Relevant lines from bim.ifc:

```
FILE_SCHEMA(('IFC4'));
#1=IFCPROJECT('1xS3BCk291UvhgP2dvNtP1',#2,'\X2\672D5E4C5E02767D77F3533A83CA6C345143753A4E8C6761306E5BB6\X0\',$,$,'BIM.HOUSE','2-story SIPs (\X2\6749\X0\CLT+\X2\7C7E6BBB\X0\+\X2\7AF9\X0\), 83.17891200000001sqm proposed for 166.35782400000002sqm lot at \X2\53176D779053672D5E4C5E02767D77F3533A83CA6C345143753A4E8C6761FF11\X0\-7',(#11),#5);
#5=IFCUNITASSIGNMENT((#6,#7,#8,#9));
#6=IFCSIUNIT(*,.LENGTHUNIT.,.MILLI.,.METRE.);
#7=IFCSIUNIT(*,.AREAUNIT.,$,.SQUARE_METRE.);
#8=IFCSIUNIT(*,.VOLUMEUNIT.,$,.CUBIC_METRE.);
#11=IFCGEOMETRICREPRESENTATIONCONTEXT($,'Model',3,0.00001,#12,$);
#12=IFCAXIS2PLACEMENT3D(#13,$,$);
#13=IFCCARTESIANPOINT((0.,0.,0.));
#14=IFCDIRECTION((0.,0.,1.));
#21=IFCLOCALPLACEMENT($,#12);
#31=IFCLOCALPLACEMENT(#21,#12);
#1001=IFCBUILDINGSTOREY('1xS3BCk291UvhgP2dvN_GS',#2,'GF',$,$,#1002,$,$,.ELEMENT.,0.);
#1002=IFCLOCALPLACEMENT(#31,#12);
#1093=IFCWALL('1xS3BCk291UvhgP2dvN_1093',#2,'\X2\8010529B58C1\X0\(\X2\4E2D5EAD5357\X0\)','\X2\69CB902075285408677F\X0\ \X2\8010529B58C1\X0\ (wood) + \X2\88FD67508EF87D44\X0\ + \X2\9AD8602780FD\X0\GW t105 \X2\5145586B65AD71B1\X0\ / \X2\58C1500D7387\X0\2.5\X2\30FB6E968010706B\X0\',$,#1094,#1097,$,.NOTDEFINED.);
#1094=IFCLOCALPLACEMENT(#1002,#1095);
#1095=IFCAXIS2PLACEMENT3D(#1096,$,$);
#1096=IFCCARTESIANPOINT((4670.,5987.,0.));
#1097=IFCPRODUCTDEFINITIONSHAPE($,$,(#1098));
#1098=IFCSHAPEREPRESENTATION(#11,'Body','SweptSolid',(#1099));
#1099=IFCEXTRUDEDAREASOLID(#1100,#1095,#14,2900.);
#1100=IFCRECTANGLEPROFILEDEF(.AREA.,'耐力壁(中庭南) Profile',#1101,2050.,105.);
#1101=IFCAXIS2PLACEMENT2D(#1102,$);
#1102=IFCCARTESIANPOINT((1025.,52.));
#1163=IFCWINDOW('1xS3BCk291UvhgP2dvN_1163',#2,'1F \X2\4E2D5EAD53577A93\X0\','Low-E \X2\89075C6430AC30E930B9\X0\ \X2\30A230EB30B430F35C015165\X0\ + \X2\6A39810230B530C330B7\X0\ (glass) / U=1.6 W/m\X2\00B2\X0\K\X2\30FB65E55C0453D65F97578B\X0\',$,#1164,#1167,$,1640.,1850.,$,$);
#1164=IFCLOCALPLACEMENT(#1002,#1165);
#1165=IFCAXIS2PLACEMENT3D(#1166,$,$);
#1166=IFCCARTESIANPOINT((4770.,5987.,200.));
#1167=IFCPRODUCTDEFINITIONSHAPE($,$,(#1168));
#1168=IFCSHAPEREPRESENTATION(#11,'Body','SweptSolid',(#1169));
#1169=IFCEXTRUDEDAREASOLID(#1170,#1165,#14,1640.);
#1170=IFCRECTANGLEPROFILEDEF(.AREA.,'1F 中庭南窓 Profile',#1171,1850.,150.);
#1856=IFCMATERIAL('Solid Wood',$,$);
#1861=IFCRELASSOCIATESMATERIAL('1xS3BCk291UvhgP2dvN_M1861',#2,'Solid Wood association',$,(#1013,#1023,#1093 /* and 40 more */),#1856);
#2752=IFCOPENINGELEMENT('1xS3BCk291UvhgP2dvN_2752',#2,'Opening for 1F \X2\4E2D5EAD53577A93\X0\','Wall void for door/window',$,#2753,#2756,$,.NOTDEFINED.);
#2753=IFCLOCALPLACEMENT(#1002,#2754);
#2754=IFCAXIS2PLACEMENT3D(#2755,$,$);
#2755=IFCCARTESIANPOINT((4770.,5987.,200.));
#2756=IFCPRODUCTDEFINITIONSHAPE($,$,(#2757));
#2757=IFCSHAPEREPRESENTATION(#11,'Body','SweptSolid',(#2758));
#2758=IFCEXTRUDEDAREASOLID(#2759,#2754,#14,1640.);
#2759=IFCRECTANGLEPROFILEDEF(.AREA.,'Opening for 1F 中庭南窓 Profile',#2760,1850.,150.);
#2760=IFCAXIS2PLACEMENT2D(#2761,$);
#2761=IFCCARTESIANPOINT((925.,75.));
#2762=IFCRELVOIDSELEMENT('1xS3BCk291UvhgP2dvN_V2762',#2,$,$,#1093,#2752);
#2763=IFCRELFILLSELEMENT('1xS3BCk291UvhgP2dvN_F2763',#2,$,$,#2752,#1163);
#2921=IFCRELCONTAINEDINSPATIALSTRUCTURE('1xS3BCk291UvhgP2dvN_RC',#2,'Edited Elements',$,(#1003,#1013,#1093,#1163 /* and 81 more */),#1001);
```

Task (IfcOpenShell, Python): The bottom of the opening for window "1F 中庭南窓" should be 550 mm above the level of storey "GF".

```python
import numpy as np
import ifcopenshell
import ifcopenshell.api.geometry
import ifcopenshell.geom
import ifcopenshell.util.element
import ifcopenshell.util.placement
import ifcopenshell.util.shape
import ifcopenshell.util.unit

model = ifcopenshell.open("bim.ifc")
unit_scale = ifcopenshell.util.unit.calculate_unit_scale(model)

window = model.by_id(1163)
opening = window.FillsVoids[0].RelatingOpeningElement
storey = ifcopenshell.util.element.get_container(window, ifc_class="IfcBuildingStorey")
level = ifcopenshell.util.placement.get_local_placement(storey.ObjectPlacement)[2, 3]

# The opening's origin need not be at the sill, so measure its lowest point.
shape = ifcopenshell.geom.create_shape(ifcopenshell.geom.settings(), opening)
bottom = ifcopenshell.util.shape.get_shape_bottom_elevation(shape, shape.geometry) / unit_scale
dz = level + 0.55 / unit_scale - bottom

shift = np.array([0.0, 0.0, dz])
# The window is not placed relative to its opening, so move both.
for product in (opening, window):
    matrix = ifcopenshell.util.placement.get_local_placement(product.ObjectPlacement)
    matrix[:3, 3] += shift
    ifcopenshell.api.geometry.edit_object_placement(model, product=product, matrix=matrix, is_si=False)

print(f"moved by {dz * unit_scale:+.3f} m")

model.write("bim_updated.ifc")
```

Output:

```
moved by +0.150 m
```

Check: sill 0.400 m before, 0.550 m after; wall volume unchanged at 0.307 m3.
